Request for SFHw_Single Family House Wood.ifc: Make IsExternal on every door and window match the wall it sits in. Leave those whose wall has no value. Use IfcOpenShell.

First a look at what the model holds.

```python
import ifcopenshell
import ifcopenshell.util.element

model = ifcopenshell.open("SFHw_Single Family House Wood.ifc")
print(model.schema)
seen = {}
for e in model.by_type("IfcDoor") + model.by_type("IfcWindow"):
    if not e.FillsVoids:
        continue
    host = e.FillsVoids[0].RelatingOpeningElement.VoidsElements[0].RelatingBuildingElement
    own = ifcopenshell.util.element.get_pset(e, f"Pset_{e.is_a()[3:].removesuffix('StandardCase')}Common", "IsExternal")
    wall = ifcopenshell.util.element.get_pset(host, "Pset_WallCommon", "IsExternal")
    seen[e.is_a(), own, wall] = seen.get((e.is_a(), own, wall), 0) + 1
for (cls, own, wall), count in sorted(seen.items(), key=str):
    print(count, cls, "IsExternal:", own, "| host wall:", wall)
```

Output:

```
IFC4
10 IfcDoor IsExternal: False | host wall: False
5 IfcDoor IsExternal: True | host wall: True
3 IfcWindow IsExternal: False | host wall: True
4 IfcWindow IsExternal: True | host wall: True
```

```python
import ifcopenshell
import ifcopenshell.api.pset
import ifcopenshell.util.element

model = ifcopenshell.open("SFHw_Single Family House Wood.ifc")

count = 0
for ifc_class, pset_name in (("IfcDoor", "Pset_DoorCommon"), ("IfcWindow", "Pset_WindowCommon")):
    for e in model.by_type(ifc_class):
        if not e.FillsVoids:
            continue
        host = e.FillsVoids[0].RelatingOpeningElement.VoidsElements[0].RelatingBuildingElement
        external = ifcopenshell.util.element.get_pset(host, "Pset_WallCommon", "IsExternal")
        if external is None or ifcopenshell.util.element.get_pset(e, pset_name, "IsExternal") == external:
            continue
        pset = ifcopenshell.api.pset.add_pset(model, product=e, name=pset_name)
        ifcopenshell.api.pset.edit_pset(model, pset=pset, properties={"IsExternal": external})
        count += 1

print(count, "updated")

model.write("SFHw_Single Family House Wood_rev.ifc")
```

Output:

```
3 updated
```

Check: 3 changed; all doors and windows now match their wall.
